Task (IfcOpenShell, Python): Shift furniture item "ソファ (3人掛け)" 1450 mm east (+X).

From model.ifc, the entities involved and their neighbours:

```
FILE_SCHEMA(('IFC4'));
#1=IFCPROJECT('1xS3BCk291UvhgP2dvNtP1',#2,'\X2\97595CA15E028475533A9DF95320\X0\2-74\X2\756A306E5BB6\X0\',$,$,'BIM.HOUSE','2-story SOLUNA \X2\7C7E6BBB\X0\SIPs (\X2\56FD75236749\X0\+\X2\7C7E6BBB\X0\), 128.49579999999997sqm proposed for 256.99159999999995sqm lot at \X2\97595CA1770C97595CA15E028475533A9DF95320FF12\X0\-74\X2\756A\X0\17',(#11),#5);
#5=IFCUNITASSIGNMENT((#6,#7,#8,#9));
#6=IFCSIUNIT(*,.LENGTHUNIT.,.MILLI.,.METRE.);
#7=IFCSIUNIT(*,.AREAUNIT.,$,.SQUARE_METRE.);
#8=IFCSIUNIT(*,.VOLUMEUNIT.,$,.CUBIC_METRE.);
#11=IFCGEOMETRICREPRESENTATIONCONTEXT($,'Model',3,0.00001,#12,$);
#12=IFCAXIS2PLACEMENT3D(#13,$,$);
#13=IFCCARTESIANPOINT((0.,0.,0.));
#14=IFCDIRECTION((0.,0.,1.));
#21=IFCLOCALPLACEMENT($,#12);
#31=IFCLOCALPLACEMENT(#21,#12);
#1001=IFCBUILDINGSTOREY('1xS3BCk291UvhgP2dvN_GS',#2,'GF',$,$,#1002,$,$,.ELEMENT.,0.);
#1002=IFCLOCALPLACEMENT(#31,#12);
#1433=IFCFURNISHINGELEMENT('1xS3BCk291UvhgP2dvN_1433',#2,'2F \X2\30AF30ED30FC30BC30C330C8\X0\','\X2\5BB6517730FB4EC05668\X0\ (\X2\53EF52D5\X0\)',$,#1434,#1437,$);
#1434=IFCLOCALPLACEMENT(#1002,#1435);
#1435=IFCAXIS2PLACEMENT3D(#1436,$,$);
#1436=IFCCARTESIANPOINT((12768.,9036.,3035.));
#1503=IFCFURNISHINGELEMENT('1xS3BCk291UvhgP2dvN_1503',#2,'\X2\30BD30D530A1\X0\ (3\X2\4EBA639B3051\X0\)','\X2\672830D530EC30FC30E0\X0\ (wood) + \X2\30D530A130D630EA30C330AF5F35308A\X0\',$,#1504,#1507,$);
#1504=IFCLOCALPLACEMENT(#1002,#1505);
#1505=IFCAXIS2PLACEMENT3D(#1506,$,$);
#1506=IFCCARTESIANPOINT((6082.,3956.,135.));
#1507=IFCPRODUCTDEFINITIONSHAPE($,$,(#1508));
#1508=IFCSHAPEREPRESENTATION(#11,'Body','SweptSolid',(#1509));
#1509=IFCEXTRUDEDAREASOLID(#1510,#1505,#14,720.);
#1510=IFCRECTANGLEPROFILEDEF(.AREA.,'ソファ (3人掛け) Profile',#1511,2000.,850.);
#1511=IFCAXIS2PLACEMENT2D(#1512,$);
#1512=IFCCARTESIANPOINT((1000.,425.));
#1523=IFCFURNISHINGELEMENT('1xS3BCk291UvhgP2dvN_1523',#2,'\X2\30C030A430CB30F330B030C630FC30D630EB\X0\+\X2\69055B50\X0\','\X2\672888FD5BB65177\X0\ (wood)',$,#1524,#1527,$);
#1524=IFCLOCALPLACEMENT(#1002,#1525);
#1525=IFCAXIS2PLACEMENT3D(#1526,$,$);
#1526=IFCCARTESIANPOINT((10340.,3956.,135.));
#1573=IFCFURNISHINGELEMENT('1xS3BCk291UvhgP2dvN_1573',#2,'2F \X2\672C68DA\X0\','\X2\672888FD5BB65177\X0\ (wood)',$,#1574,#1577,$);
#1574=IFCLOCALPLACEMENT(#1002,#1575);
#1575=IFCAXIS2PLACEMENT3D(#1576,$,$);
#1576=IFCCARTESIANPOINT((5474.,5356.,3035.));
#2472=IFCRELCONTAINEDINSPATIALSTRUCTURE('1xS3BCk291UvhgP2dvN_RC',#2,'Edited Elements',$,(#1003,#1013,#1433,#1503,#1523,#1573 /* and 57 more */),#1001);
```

```python
import ifcopenshell
import ifcopenshell.api.geometry
import ifcopenshell.util.placement
import ifcopenshell.util.unit

model = ifcopenshell.open("model.ifc")
unit_scale = ifcopenshell.util.unit.calculate_unit_scale(model)

item = model.by_guid("1xS3BCk291UvhgP2dvN_1503")
matrix = ifcopenshell.util.placement.get_local_placement(item.ObjectPlacement)
matrix[0, 3] += 1.45 / unit_scale
ifcopenshell.api.geometry.edit_object_placement(model, product=item, matrix=matrix, is_si=False)

print(ifcopenshell.util.placement.get_local_placement(item.ObjectPlacement).round(3) + 0.0)

model.write("model_rev.ifc")
```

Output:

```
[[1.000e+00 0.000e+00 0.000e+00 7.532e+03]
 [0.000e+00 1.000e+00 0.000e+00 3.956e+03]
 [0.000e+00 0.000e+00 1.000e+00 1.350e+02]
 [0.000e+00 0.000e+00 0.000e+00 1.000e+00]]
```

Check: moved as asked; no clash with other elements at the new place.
